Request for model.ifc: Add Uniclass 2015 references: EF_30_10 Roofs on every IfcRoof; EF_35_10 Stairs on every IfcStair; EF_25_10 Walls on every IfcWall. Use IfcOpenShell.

First a look at what the model holds.

```python
import ifcopenshell

model = ifcopenshell.open("model.ifc")
print(model.schema)
print("classifications:", [c.Name for c in model.by_type("IfcClassification")])
for ifc_class in ("IfcDoor", "IfcRoof", "IfcStair", "IfcWall", "IfcWindow"):
    print(ifc_class, len(model.by_type(ifc_class)))
```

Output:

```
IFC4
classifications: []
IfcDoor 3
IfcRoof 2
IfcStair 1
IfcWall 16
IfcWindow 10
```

```python
import ifcopenshell
import ifcopenshell.api.classification

model = ifcopenshell.open("model.ifc")

system = ifcopenshell.api.classification.add_classification(model, classification="Uniclass 2015")

codes = {
    "IfcRoof": ("EF_30_10", "Roofs"),
    "IfcStair": ("EF_35_10", "Stairs"),
    "IfcWall": ("EF_25_10", "Walls"),
}
for ifc_class, (code, name) in codes.items():
    products = model.by_type(ifc_class)
    ifcopenshell.api.classification.add_reference(
        model, products=products, classification=system, identification=code, name=name
    )
    print(code, len(products))

model.write("model_updated.ifc")
```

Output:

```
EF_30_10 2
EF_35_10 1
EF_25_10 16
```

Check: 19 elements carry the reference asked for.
